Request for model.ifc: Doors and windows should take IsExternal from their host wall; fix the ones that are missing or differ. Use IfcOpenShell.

First a look at what the model holds.

```python
import ifcopenshell
import ifcopenshell.util.element

model = ifcopenshell.open("model.ifc")
print(model.schema)
seen = {}
for e in model.by_type("IfcDoor") + model.by_type("IfcWindow"):
    if not e.FillsVoids:
        continue
    host = e.FillsVoids[0].RelatingOpeningElement.VoidsElements[0].RelatingBuildingElement
    own = ifcopenshell.util.element.get_pset(e, f"Pset_{e.is_a()[3:].removesuffix('StandardCase')}Common", "IsExternal")
    wall = ifcopenshell.util.element.get_pset(host, "Pset_WallCommon", "IsExternal")
    seen[e.is_a(), own, wall] = seen.get((e.is_a(), own, wall), 0) + 1
for (cls, own, wall), count in sorted(seen.items(), key=str):
    print(count, cls, "IsExternal:", own, "| host wall:", wall)
```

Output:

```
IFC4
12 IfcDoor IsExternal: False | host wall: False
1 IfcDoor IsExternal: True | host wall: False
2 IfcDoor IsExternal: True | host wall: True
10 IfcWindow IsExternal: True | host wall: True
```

```python
import ifcopenshell
import ifcopenshell.api.pset
import ifcopenshell.util.element

model = ifcopenshell.open("model.ifc")

count = 0
for ifc_class, pset_name in (("IfcDoor", "Pset_DoorCommon"), ("IfcWindow", "Pset_WindowCommon")):
    for e in model.by_type(ifc_class):
        if not e.FillsVoids:
            continue
        host = e.FillsVoids[0].RelatingOpeningElement.VoidsElements[0].RelatingBuildingElement
        external = ifcopenshell.util.element.get_pset(host, "Pset_WallCommon", "IsExternal")
        if external is None or ifcopenshell.util.element.get_pset(e, pset_name, "IsExternal") == external:
            continue
        pset = ifcopenshell.api.pset.add_pset(model, product=e, name=pset_name)
        ifcopenshell.api.pset.edit_pset(model, pset=pset, properties={"IsExternal": external})
        count += 1

print(count, "updated")

model.write("model_rev.ifc")
```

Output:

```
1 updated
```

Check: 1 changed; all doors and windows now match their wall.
